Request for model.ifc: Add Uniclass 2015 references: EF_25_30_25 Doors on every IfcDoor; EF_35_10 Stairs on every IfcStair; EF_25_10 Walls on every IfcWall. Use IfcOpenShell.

First a look at what the model holds.

```python
import ifcopenshell

model = ifcopenshell.open("model.ifc")
print(model.schema)
print("classifications:", [c.Name for c in model.by_type("IfcClassification")])
for ifc_class in ("IfcDoor", "IfcRoof", "IfcStair", "IfcWall", "IfcWindow"):
    print(ifc_class, len(model.by_type(ifc_class)))
```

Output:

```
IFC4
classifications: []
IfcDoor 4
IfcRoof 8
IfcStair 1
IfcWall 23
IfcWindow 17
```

```python
import ifcopenshell
import ifcopenshell.api.classification

model = ifcopenshell.open("model.ifc")

system = ifcopenshell.api.classification.add_classification(model, classification="Uniclass 2015")

codes = {
    "IfcDoor": ("EF_25_30_25", "Doors"),
    "IfcStair": ("EF_35_10", "Stairs"),
    "IfcWall": ("EF_25_10", "Walls"),
}
for ifc_class, (code, name) in codes.items():
    products = model.by_type(ifc_class)
    ifcopenshell.api.classification.add_reference(
        model, products=products, classification=system, identification=code, name=name
    )
    print(code, len(products))

model.write("model_rev.ifc")
```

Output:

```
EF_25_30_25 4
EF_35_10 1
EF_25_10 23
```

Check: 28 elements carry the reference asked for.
